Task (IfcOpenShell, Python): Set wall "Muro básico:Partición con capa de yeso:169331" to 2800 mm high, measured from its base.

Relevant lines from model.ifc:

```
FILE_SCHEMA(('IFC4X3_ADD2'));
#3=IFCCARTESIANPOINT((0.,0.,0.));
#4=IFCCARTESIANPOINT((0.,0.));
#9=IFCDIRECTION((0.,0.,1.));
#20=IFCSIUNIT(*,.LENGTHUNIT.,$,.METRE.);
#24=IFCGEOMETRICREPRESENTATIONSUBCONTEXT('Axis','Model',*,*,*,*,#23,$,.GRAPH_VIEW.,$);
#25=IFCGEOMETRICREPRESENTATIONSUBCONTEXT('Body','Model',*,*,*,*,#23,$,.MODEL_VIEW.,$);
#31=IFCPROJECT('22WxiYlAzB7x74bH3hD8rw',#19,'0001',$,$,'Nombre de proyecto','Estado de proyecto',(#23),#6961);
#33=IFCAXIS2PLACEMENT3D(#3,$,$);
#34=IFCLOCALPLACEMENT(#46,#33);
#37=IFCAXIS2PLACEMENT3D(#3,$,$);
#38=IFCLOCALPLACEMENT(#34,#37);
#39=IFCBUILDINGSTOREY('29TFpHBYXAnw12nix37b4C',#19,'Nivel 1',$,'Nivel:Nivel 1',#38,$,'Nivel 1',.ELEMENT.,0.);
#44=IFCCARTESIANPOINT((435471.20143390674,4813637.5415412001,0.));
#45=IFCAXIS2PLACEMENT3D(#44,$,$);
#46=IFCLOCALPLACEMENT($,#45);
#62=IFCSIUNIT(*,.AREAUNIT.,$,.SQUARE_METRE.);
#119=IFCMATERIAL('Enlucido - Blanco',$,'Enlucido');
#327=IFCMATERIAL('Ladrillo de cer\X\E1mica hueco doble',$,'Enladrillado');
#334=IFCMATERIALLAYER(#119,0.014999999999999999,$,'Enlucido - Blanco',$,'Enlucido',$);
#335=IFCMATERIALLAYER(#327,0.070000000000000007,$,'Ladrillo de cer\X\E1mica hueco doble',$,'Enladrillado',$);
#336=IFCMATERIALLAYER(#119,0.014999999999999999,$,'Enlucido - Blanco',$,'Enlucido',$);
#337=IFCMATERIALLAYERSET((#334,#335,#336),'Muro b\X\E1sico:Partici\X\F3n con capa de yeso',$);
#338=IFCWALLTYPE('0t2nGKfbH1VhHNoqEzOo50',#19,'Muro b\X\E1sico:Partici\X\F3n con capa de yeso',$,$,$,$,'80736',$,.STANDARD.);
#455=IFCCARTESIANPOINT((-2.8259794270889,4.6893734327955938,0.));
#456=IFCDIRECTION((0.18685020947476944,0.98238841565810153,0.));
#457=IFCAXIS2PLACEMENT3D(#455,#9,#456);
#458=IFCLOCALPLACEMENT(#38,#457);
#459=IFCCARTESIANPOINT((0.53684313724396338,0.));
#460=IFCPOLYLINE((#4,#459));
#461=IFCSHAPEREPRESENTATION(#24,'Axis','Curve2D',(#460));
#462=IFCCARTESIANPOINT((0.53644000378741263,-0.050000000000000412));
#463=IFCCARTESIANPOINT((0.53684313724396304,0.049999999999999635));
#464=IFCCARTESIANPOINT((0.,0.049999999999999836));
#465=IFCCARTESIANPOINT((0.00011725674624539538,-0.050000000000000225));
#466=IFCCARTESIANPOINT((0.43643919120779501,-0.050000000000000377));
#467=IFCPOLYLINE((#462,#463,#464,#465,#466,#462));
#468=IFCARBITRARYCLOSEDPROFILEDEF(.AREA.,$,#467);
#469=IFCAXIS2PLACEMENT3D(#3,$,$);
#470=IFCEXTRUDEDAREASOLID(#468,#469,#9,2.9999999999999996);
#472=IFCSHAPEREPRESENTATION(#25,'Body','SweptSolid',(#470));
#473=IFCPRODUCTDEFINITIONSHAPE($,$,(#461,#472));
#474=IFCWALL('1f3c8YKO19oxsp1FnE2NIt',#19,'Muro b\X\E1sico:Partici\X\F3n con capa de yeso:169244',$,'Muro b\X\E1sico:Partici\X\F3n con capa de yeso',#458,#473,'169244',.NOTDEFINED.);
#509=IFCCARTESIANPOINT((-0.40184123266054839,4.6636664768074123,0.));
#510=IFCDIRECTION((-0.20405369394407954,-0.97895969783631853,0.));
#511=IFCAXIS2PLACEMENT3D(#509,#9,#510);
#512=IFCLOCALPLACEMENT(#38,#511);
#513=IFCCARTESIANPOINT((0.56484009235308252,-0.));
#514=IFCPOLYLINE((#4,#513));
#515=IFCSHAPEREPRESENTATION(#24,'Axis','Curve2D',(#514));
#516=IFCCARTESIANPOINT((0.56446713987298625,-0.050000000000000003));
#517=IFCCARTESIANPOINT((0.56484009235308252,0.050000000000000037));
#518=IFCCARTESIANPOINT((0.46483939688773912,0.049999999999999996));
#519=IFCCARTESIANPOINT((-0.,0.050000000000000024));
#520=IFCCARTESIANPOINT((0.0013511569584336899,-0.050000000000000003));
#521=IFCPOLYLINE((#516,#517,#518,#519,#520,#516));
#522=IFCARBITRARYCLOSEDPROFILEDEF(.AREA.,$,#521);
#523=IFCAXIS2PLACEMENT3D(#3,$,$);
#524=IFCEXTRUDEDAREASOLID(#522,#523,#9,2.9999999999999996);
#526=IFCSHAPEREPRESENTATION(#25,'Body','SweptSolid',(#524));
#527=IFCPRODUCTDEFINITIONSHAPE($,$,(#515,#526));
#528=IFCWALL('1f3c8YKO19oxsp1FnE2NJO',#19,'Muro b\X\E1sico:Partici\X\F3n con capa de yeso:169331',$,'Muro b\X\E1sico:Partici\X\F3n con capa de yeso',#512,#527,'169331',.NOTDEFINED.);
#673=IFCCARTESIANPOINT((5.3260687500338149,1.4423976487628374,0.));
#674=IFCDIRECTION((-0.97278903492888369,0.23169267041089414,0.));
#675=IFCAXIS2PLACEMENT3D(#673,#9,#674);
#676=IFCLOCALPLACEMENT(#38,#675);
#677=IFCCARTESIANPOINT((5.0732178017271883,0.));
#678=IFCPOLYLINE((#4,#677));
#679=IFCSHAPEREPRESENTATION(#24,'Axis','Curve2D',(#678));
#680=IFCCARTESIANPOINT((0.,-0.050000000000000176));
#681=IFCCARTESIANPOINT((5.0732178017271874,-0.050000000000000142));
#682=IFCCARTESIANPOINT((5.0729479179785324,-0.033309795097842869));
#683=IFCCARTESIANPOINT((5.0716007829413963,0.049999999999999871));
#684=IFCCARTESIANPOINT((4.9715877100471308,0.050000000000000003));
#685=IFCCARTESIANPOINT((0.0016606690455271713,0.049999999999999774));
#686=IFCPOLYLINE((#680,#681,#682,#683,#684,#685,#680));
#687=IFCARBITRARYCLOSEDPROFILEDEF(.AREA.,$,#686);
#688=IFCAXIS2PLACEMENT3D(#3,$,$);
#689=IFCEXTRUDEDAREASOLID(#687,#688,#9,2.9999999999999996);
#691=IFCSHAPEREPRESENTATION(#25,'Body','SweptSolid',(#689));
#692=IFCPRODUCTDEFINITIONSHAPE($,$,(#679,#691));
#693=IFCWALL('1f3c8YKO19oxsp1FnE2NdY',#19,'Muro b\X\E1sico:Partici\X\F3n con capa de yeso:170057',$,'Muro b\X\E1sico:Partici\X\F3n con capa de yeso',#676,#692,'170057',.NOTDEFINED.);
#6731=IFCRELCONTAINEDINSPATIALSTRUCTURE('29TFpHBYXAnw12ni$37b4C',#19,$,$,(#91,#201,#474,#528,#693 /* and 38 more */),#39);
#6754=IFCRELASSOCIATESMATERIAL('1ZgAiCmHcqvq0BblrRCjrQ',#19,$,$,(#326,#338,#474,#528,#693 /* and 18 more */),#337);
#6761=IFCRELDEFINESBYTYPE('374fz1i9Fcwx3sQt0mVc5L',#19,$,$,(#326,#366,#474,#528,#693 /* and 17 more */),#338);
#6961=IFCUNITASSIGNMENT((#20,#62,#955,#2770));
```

```python
import ifcopenshell
import ifcopenshell.geom
import ifcopenshell.util.representation
import ifcopenshell.util.shape
import ifcopenshell.util.unit

model = ifcopenshell.open("model.ifc")
unit_scale = ifcopenshell.util.unit.calculate_unit_scale(model)
settings = ifcopenshell.geom.settings()


def volume(element):
    """Net volume in cubic metres, openings subtracted."""
    shape = ifcopenshell.geom.create_shape(settings, element)
    return ifcopenshell.util.shape.get_volume(shape.geometry)


wall = model.by_guid("1f3c8YKO19oxsp1FnE2NJO")
before = volume(wall)

body = ifcopenshell.util.representation.get_representation(wall, "Model", "Body")
solid = body.Items[0]
old_height = solid.Depth
solid.Depth = 2.8 / unit_scale
after = volume(wall)

print(f"height {old_height:g} -> {solid.Depth:g}, volume {before:.3f} -> {after:.3f} m3")

model.write("model_v2.ifc")
```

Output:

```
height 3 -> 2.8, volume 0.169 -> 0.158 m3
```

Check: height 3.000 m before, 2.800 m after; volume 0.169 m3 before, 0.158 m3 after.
